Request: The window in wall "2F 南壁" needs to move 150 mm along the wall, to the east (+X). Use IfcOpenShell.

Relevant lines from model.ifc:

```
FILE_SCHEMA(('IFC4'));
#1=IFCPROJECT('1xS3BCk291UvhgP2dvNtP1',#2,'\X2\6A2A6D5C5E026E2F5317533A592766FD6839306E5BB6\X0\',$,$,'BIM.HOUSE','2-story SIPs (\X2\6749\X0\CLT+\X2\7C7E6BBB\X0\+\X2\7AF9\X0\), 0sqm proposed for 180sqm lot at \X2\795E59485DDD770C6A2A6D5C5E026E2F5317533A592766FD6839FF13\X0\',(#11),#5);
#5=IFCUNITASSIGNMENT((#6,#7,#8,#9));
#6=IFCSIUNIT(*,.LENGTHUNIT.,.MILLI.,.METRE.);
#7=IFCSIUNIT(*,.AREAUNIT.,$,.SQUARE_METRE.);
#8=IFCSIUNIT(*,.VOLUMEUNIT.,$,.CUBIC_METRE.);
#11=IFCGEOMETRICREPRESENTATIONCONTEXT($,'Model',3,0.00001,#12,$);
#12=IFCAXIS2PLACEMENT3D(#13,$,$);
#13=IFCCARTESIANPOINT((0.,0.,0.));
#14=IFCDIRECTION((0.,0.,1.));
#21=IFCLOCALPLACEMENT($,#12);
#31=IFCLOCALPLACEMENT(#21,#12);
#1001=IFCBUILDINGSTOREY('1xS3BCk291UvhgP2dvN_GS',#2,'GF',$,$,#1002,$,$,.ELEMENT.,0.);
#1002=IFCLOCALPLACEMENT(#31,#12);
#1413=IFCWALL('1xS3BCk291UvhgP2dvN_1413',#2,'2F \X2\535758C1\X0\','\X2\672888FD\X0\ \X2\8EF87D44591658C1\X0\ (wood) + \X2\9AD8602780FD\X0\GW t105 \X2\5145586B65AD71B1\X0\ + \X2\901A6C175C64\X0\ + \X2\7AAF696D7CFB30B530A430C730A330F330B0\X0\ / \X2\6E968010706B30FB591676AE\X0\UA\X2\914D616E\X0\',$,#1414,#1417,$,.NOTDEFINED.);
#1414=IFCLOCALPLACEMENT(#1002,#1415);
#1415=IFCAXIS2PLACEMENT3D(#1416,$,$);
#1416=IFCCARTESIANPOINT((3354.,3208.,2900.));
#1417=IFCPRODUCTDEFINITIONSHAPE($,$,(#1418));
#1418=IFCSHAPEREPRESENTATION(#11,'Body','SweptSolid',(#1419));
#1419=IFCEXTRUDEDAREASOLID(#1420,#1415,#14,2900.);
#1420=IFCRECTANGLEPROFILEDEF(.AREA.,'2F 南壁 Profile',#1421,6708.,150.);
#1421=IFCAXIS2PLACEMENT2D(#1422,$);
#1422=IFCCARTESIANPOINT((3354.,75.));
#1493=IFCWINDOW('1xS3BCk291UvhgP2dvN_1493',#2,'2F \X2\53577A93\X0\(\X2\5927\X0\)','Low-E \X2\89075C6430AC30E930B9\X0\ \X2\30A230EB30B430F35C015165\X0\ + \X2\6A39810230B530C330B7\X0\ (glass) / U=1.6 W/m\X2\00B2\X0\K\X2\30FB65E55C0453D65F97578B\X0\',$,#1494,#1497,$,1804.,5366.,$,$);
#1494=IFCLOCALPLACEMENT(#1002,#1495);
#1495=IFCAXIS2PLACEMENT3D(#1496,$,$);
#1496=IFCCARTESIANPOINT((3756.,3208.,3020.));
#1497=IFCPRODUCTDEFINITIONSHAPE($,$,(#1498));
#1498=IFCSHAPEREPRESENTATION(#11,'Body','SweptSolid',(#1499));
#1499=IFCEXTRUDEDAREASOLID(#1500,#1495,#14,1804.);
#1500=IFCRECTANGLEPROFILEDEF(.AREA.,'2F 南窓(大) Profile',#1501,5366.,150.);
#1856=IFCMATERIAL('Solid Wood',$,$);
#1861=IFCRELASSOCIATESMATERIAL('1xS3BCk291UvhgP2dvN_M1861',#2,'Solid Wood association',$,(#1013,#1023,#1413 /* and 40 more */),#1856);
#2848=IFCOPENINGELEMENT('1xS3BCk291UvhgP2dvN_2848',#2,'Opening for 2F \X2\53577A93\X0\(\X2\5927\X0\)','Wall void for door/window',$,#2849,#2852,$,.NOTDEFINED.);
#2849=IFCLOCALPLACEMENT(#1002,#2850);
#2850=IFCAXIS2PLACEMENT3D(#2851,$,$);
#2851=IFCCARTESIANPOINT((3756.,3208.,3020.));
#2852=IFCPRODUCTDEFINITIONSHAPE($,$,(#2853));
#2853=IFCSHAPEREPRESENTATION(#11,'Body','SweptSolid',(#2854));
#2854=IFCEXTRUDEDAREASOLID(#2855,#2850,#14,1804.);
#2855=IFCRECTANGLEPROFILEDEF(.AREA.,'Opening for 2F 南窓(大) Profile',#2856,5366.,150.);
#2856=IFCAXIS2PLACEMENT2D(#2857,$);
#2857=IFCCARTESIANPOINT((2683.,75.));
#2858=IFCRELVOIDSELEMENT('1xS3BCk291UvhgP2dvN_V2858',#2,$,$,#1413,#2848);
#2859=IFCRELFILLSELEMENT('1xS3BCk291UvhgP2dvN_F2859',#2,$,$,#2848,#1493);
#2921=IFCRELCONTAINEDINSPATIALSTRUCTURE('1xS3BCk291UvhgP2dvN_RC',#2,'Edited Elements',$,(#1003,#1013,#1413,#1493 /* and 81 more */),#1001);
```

```python
import ifcopenshell
import ifcopenshell.api.geometry
import ifcopenshell.util.placement

model = ifcopenshell.open("model.ifc")

window = model.by_guid("1xS3BCk291UvhgP2dvN_1493")
opening = window.FillsVoids[0].RelatingOpeningElement
wall = opening.VoidsElements[0].RelatingBuildingElement

wall_matrix = ifcopenshell.util.placement.get_local_placement(wall.ObjectPlacement)
shift = wall_matrix[:3, 0] * 150.0
before = ifcopenshell.util.placement.get_local_placement(window.ObjectPlacement)[:3, 3].copy()

# The window is not placed relative to its opening, so move both.
for product in (opening, window):
    matrix = ifcopenshell.util.placement.get_local_placement(product.ObjectPlacement)
    matrix[:3, 3] += shift
    ifcopenshell.api.geometry.edit_object_placement(model, product=product, matrix=matrix, is_si=False)

after = ifcopenshell.util.placement.get_local_placement(window.ObjectPlacement)[:3, 3]
print("window moved by", (after - before).round(3) + 0.0)

model.write("model_edited.ifc")
```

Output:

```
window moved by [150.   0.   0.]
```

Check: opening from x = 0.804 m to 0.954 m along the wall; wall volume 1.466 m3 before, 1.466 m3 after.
